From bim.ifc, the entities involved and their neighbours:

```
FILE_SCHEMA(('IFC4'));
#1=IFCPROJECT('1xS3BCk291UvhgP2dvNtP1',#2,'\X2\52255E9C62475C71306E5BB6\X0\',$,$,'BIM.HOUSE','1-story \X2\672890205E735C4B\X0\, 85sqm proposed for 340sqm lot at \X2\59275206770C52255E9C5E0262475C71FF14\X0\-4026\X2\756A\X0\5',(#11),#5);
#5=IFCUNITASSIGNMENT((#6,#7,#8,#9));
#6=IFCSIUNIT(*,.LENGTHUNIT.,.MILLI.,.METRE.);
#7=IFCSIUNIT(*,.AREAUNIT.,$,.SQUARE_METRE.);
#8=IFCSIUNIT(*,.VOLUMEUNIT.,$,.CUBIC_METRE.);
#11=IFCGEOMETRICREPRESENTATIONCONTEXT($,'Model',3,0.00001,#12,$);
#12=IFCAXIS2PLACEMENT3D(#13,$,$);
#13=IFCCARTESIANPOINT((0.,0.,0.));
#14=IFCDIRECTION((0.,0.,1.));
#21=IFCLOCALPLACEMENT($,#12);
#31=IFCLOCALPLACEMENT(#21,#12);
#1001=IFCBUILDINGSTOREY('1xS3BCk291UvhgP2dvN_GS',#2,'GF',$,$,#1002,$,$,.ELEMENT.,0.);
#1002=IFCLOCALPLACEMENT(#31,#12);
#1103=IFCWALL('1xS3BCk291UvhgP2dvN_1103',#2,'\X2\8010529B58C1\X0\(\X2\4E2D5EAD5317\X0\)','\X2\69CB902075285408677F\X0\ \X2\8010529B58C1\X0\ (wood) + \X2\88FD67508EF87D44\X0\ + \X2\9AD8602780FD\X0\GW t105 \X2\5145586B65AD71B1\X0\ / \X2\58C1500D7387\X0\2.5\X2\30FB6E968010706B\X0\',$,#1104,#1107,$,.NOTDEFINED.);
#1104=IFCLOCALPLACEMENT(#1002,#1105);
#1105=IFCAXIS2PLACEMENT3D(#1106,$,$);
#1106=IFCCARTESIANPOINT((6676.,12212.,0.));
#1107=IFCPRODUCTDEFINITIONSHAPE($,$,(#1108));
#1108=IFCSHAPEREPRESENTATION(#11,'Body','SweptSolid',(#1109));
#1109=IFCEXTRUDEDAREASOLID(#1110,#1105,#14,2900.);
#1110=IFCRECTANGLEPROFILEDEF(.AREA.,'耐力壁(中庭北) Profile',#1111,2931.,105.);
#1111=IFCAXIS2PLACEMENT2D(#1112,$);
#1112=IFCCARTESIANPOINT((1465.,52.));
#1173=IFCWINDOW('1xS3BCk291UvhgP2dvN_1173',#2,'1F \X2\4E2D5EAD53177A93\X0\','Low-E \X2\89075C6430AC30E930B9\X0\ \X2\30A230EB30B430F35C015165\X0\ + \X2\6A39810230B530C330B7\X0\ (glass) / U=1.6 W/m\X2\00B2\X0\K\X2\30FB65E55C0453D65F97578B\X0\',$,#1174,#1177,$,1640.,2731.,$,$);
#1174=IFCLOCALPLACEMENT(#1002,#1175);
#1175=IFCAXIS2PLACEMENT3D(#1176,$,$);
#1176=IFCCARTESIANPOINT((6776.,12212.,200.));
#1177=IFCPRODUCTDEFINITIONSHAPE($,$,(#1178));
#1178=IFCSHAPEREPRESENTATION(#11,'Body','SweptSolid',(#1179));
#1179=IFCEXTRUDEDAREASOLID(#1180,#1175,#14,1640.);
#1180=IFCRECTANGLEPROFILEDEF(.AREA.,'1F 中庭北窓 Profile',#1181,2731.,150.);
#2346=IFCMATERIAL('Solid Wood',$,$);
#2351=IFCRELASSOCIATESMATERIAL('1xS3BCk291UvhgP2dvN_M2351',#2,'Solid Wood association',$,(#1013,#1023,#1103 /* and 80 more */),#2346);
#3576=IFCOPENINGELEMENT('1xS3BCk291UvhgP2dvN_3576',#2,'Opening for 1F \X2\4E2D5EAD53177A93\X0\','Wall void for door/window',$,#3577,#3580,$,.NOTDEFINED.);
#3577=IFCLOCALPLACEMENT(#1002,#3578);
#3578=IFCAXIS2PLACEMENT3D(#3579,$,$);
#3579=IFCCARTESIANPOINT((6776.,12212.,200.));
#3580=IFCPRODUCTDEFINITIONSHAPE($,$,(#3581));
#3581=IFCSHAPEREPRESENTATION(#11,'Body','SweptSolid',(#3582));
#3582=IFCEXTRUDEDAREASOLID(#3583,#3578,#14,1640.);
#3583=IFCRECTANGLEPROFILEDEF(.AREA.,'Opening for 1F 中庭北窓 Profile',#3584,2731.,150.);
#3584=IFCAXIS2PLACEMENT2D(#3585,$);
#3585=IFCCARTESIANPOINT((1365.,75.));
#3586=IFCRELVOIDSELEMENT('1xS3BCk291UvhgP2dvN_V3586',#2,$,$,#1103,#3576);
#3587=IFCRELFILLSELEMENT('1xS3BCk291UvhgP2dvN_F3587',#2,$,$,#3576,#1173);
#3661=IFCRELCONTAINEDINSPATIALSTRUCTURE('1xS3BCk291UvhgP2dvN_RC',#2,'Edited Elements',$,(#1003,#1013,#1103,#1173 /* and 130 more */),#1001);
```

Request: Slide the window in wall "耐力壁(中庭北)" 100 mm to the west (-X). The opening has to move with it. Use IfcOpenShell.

```python
import ifcopenshell
import ifcopenshell.api.geometry
import ifcopenshell.util.placement
import ifcopenshell.util.unit

model = ifcopenshell.open("bim.ifc")
unit_scale = ifcopenshell.util.unit.calculate_unit_scale(model)

window = model.by_id(1173)
opening = window.FillsVoids[0].RelatingOpeningElement
wall = opening.VoidsElements[0].RelatingBuildingElement

wall_matrix = ifcopenshell.util.placement.get_local_placement(wall.ObjectPlacement)
shift = wall_matrix[:3, 0] * -0.1 / unit_scale
before = ifcopenshell.util.placement.get_local_placement(window.ObjectPlacement)[:3, 3].copy()

# The window is not placed relative to its opening, so move both.
for product in (opening, window):
    matrix = ifcopenshell.util.placement.get_local_placement(product.ObjectPlacement)
    matrix[:3, 3] += shift
    ifcopenshell.api.geometry.edit_object_placement(model, product=product, matrix=matrix, is_si=False)

after = ifcopenshell.util.placement.get_local_placement(window.ObjectPlacement)[:3, 3]
print("window moved by", (after - before).round(3) + 0.0)

model.write("bim_v2.ifc")
```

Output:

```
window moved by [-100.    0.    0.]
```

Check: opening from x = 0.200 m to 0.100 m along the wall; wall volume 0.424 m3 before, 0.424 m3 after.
